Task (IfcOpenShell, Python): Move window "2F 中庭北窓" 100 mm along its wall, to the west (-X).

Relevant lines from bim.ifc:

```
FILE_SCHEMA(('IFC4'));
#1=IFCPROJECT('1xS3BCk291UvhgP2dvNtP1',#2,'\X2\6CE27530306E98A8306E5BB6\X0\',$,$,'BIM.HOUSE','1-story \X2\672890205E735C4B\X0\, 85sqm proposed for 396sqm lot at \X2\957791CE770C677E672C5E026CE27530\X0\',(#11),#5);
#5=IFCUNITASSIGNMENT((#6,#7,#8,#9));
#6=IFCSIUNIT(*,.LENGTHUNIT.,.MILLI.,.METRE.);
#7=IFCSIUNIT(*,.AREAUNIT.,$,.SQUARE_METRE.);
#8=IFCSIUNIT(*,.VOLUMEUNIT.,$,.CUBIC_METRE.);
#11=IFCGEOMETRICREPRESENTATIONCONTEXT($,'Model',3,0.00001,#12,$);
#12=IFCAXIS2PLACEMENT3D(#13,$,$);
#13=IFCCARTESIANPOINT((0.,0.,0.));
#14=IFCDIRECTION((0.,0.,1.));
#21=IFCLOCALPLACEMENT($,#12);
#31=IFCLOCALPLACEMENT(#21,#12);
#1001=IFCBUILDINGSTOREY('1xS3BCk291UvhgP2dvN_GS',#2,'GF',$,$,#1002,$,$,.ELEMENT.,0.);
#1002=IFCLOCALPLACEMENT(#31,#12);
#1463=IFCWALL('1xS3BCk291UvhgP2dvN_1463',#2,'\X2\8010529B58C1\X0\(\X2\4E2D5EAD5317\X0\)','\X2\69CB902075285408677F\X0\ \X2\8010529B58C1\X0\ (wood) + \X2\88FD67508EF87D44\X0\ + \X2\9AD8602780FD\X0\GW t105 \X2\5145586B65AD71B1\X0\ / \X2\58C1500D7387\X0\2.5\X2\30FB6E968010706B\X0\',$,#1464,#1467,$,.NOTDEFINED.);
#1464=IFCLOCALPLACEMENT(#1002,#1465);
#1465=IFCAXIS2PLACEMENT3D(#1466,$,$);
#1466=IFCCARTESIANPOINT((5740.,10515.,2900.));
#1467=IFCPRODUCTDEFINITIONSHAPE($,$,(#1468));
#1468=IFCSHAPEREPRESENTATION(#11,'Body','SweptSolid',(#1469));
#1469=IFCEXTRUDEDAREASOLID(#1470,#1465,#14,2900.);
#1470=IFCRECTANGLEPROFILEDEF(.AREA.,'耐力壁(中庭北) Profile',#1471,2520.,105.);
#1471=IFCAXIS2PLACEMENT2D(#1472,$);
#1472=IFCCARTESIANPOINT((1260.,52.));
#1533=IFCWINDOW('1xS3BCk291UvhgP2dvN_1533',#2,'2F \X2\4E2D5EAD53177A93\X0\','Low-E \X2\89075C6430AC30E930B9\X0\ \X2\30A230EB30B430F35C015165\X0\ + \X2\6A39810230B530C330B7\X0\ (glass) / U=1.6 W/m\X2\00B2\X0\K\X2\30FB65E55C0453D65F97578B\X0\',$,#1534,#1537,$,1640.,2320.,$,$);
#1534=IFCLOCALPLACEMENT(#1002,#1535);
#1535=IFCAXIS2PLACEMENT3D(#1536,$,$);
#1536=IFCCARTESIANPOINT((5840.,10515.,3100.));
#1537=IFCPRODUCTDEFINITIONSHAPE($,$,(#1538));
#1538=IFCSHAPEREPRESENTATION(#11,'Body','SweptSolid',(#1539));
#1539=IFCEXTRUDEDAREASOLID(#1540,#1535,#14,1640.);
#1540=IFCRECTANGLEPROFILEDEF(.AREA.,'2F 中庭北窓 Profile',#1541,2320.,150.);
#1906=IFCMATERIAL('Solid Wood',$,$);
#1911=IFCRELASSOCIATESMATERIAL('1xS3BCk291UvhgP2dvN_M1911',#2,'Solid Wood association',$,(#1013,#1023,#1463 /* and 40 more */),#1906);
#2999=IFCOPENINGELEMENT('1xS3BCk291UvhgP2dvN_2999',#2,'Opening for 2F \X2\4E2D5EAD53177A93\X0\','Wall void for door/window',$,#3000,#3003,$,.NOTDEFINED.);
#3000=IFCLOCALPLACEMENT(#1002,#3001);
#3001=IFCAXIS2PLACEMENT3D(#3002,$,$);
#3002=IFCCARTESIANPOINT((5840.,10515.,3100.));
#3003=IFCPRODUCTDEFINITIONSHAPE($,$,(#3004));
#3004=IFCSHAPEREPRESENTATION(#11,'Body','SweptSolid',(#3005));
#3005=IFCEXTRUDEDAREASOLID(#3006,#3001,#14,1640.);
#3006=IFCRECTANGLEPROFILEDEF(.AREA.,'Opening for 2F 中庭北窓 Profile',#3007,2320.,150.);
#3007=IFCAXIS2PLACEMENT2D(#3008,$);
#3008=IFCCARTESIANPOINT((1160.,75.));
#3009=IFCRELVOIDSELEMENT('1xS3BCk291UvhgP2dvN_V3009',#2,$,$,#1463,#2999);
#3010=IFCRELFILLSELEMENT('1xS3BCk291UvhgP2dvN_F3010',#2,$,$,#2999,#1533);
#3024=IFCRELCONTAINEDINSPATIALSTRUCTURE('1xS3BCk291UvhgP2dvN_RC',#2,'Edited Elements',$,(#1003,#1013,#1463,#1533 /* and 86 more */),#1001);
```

```python
import ifcopenshell
import ifcopenshell.api.geometry
import ifcopenshell.util.placement

model = ifcopenshell.open("bim.ifc")

window = model.by_id(1533)
opening = window.FillsVoids[0].RelatingOpeningElement
wall = opening.VoidsElements[0].RelatingBuildingElement

wall_matrix = ifcopenshell.util.placement.get_local_placement(wall.ObjectPlacement)
shift = wall_matrix[:3, 0] * -100.0
before = ifcopenshell.util.placement.get_local_placement(window.ObjectPlacement)[:3, 3].copy()

# The window is not placed relative to its opening, so move both.
for product in (opening, window):
    matrix = ifcopenshell.util.placement.get_local_placement(product.ObjectPlacement)
    matrix[:3, 3] += shift
    ifcopenshell.api.geometry.edit_object_placement(model, product=product, matrix=matrix, is_si=False)

after = ifcopenshell.util.placement.get_local_placement(window.ObjectPlacement)[:3, 3]
print("window moved by", (after - before).round(3) + 0.0)

model.write("bim-out.ifc")
```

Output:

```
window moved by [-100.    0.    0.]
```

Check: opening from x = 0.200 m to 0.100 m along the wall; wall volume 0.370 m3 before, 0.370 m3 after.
